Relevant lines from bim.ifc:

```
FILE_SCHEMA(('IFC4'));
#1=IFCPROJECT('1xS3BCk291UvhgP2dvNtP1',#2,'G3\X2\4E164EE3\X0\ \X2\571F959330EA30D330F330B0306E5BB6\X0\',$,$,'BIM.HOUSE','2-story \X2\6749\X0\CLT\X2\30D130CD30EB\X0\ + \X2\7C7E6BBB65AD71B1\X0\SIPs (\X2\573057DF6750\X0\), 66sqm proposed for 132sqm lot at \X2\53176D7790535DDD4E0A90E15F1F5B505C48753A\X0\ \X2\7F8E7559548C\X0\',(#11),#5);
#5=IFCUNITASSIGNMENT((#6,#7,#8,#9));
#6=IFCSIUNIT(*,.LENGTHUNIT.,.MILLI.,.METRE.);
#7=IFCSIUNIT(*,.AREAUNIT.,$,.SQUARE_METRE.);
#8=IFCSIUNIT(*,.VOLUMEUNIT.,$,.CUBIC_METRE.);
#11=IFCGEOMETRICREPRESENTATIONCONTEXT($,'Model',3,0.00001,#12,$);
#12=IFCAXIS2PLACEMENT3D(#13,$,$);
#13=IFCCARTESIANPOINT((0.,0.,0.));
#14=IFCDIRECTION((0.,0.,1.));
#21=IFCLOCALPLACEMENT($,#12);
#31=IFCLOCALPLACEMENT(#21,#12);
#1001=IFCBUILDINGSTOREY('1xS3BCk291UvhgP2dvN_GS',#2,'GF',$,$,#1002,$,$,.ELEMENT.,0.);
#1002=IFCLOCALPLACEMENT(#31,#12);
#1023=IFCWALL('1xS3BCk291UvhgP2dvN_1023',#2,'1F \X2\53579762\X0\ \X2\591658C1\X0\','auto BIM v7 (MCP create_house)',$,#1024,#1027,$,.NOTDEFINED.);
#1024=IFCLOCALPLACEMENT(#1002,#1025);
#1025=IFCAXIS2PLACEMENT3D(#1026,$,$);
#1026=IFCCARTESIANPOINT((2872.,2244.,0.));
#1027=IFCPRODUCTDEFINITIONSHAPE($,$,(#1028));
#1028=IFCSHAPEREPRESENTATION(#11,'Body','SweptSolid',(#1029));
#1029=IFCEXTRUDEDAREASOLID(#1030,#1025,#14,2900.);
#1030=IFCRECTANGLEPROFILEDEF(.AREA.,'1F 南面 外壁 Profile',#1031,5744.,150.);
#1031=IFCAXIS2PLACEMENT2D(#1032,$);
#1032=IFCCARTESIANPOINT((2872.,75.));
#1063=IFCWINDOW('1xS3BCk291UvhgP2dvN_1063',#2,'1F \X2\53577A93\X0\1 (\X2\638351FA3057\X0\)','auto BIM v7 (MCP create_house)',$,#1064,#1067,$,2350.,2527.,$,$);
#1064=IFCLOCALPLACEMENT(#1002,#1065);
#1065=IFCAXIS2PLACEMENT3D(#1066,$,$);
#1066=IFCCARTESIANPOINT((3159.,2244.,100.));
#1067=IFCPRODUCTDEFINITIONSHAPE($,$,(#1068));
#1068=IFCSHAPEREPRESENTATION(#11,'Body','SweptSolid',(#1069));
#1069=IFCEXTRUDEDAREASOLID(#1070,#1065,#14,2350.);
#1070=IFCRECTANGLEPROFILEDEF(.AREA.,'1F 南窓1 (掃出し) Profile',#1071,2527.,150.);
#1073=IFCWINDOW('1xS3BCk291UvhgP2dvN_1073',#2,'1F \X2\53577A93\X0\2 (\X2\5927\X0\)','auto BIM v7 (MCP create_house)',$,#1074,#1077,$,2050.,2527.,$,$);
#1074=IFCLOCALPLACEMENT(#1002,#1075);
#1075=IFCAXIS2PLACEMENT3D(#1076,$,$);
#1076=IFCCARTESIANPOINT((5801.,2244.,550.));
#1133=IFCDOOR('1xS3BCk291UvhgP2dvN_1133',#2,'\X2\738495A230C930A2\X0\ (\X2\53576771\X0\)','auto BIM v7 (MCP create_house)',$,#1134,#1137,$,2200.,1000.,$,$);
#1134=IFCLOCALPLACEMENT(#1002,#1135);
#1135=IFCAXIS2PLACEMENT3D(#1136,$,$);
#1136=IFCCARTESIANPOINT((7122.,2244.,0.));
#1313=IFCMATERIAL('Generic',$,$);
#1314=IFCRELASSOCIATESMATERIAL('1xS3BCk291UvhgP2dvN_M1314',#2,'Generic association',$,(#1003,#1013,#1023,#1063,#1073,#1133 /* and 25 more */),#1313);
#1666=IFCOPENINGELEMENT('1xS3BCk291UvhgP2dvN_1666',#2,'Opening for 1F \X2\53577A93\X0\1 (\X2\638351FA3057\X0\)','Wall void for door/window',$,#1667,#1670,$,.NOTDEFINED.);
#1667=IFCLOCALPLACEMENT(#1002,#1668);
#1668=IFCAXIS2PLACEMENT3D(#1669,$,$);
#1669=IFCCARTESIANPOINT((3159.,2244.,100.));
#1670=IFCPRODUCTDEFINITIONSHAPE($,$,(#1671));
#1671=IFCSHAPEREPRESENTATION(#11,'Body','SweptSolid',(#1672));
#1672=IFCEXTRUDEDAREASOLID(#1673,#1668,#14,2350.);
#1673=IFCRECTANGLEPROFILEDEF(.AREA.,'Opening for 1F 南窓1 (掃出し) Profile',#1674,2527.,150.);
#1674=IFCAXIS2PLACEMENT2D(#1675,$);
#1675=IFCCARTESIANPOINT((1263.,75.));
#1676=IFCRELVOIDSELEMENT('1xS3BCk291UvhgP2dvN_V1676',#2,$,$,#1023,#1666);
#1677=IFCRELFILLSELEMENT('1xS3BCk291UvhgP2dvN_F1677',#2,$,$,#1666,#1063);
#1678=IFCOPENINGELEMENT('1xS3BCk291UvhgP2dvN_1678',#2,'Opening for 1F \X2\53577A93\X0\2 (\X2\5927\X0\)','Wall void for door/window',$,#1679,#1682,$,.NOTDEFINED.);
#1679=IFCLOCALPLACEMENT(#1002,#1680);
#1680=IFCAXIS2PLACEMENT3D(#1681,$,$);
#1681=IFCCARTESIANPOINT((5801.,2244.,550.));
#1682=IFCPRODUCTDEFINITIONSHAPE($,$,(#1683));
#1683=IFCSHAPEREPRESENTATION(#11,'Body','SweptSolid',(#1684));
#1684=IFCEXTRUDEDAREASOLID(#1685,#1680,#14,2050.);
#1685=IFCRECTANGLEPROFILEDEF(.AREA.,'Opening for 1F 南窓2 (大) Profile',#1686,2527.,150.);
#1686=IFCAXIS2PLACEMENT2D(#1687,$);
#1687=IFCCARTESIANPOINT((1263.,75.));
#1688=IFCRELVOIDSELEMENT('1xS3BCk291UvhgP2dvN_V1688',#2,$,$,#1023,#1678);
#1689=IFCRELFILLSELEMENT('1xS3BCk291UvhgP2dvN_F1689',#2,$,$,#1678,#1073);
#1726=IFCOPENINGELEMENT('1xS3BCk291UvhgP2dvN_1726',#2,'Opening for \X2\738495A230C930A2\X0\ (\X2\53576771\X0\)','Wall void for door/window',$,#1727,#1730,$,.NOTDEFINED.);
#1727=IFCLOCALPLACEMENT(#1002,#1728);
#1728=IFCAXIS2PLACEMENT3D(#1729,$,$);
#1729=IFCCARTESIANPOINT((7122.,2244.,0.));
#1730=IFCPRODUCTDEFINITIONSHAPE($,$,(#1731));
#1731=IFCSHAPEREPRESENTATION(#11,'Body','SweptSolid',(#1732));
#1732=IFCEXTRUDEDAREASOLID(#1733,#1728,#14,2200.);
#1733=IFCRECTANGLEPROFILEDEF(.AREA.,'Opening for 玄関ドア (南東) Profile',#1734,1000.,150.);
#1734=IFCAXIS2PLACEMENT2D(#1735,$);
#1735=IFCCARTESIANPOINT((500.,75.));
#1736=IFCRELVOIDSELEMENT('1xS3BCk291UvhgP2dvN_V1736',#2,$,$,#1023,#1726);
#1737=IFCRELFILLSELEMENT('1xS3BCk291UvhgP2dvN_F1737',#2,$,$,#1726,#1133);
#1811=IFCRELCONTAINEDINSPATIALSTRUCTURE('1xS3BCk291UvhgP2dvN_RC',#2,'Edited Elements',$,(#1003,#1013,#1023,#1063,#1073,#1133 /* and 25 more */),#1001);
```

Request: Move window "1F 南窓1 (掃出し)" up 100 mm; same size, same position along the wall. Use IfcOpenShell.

```python
import numpy as np
import ifcopenshell
import ifcopenshell.api.geometry
import ifcopenshell.util.placement
import ifcopenshell.util.unit

model = ifcopenshell.open("bim.ifc")
unit_scale = ifcopenshell.util.unit.calculate_unit_scale(model)

window = model.by_id(1063)
opening = window.FillsVoids[0].RelatingOpeningElement
dz = 100.0

shift = np.array([0.0, 0.0, dz])
# The window is not placed relative to its opening, so move both.
for product in (opening, window):
    matrix = ifcopenshell.util.placement.get_local_placement(product.ObjectPlacement)
    matrix[:3, 3] += shift
    ifcopenshell.api.geometry.edit_object_placement(model, product=product, matrix=matrix, is_si=False)

print(f"moved by {dz * unit_scale:+.3f} m")

model.write("bim_updated.ifc")
```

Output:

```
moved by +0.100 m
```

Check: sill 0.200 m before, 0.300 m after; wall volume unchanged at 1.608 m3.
